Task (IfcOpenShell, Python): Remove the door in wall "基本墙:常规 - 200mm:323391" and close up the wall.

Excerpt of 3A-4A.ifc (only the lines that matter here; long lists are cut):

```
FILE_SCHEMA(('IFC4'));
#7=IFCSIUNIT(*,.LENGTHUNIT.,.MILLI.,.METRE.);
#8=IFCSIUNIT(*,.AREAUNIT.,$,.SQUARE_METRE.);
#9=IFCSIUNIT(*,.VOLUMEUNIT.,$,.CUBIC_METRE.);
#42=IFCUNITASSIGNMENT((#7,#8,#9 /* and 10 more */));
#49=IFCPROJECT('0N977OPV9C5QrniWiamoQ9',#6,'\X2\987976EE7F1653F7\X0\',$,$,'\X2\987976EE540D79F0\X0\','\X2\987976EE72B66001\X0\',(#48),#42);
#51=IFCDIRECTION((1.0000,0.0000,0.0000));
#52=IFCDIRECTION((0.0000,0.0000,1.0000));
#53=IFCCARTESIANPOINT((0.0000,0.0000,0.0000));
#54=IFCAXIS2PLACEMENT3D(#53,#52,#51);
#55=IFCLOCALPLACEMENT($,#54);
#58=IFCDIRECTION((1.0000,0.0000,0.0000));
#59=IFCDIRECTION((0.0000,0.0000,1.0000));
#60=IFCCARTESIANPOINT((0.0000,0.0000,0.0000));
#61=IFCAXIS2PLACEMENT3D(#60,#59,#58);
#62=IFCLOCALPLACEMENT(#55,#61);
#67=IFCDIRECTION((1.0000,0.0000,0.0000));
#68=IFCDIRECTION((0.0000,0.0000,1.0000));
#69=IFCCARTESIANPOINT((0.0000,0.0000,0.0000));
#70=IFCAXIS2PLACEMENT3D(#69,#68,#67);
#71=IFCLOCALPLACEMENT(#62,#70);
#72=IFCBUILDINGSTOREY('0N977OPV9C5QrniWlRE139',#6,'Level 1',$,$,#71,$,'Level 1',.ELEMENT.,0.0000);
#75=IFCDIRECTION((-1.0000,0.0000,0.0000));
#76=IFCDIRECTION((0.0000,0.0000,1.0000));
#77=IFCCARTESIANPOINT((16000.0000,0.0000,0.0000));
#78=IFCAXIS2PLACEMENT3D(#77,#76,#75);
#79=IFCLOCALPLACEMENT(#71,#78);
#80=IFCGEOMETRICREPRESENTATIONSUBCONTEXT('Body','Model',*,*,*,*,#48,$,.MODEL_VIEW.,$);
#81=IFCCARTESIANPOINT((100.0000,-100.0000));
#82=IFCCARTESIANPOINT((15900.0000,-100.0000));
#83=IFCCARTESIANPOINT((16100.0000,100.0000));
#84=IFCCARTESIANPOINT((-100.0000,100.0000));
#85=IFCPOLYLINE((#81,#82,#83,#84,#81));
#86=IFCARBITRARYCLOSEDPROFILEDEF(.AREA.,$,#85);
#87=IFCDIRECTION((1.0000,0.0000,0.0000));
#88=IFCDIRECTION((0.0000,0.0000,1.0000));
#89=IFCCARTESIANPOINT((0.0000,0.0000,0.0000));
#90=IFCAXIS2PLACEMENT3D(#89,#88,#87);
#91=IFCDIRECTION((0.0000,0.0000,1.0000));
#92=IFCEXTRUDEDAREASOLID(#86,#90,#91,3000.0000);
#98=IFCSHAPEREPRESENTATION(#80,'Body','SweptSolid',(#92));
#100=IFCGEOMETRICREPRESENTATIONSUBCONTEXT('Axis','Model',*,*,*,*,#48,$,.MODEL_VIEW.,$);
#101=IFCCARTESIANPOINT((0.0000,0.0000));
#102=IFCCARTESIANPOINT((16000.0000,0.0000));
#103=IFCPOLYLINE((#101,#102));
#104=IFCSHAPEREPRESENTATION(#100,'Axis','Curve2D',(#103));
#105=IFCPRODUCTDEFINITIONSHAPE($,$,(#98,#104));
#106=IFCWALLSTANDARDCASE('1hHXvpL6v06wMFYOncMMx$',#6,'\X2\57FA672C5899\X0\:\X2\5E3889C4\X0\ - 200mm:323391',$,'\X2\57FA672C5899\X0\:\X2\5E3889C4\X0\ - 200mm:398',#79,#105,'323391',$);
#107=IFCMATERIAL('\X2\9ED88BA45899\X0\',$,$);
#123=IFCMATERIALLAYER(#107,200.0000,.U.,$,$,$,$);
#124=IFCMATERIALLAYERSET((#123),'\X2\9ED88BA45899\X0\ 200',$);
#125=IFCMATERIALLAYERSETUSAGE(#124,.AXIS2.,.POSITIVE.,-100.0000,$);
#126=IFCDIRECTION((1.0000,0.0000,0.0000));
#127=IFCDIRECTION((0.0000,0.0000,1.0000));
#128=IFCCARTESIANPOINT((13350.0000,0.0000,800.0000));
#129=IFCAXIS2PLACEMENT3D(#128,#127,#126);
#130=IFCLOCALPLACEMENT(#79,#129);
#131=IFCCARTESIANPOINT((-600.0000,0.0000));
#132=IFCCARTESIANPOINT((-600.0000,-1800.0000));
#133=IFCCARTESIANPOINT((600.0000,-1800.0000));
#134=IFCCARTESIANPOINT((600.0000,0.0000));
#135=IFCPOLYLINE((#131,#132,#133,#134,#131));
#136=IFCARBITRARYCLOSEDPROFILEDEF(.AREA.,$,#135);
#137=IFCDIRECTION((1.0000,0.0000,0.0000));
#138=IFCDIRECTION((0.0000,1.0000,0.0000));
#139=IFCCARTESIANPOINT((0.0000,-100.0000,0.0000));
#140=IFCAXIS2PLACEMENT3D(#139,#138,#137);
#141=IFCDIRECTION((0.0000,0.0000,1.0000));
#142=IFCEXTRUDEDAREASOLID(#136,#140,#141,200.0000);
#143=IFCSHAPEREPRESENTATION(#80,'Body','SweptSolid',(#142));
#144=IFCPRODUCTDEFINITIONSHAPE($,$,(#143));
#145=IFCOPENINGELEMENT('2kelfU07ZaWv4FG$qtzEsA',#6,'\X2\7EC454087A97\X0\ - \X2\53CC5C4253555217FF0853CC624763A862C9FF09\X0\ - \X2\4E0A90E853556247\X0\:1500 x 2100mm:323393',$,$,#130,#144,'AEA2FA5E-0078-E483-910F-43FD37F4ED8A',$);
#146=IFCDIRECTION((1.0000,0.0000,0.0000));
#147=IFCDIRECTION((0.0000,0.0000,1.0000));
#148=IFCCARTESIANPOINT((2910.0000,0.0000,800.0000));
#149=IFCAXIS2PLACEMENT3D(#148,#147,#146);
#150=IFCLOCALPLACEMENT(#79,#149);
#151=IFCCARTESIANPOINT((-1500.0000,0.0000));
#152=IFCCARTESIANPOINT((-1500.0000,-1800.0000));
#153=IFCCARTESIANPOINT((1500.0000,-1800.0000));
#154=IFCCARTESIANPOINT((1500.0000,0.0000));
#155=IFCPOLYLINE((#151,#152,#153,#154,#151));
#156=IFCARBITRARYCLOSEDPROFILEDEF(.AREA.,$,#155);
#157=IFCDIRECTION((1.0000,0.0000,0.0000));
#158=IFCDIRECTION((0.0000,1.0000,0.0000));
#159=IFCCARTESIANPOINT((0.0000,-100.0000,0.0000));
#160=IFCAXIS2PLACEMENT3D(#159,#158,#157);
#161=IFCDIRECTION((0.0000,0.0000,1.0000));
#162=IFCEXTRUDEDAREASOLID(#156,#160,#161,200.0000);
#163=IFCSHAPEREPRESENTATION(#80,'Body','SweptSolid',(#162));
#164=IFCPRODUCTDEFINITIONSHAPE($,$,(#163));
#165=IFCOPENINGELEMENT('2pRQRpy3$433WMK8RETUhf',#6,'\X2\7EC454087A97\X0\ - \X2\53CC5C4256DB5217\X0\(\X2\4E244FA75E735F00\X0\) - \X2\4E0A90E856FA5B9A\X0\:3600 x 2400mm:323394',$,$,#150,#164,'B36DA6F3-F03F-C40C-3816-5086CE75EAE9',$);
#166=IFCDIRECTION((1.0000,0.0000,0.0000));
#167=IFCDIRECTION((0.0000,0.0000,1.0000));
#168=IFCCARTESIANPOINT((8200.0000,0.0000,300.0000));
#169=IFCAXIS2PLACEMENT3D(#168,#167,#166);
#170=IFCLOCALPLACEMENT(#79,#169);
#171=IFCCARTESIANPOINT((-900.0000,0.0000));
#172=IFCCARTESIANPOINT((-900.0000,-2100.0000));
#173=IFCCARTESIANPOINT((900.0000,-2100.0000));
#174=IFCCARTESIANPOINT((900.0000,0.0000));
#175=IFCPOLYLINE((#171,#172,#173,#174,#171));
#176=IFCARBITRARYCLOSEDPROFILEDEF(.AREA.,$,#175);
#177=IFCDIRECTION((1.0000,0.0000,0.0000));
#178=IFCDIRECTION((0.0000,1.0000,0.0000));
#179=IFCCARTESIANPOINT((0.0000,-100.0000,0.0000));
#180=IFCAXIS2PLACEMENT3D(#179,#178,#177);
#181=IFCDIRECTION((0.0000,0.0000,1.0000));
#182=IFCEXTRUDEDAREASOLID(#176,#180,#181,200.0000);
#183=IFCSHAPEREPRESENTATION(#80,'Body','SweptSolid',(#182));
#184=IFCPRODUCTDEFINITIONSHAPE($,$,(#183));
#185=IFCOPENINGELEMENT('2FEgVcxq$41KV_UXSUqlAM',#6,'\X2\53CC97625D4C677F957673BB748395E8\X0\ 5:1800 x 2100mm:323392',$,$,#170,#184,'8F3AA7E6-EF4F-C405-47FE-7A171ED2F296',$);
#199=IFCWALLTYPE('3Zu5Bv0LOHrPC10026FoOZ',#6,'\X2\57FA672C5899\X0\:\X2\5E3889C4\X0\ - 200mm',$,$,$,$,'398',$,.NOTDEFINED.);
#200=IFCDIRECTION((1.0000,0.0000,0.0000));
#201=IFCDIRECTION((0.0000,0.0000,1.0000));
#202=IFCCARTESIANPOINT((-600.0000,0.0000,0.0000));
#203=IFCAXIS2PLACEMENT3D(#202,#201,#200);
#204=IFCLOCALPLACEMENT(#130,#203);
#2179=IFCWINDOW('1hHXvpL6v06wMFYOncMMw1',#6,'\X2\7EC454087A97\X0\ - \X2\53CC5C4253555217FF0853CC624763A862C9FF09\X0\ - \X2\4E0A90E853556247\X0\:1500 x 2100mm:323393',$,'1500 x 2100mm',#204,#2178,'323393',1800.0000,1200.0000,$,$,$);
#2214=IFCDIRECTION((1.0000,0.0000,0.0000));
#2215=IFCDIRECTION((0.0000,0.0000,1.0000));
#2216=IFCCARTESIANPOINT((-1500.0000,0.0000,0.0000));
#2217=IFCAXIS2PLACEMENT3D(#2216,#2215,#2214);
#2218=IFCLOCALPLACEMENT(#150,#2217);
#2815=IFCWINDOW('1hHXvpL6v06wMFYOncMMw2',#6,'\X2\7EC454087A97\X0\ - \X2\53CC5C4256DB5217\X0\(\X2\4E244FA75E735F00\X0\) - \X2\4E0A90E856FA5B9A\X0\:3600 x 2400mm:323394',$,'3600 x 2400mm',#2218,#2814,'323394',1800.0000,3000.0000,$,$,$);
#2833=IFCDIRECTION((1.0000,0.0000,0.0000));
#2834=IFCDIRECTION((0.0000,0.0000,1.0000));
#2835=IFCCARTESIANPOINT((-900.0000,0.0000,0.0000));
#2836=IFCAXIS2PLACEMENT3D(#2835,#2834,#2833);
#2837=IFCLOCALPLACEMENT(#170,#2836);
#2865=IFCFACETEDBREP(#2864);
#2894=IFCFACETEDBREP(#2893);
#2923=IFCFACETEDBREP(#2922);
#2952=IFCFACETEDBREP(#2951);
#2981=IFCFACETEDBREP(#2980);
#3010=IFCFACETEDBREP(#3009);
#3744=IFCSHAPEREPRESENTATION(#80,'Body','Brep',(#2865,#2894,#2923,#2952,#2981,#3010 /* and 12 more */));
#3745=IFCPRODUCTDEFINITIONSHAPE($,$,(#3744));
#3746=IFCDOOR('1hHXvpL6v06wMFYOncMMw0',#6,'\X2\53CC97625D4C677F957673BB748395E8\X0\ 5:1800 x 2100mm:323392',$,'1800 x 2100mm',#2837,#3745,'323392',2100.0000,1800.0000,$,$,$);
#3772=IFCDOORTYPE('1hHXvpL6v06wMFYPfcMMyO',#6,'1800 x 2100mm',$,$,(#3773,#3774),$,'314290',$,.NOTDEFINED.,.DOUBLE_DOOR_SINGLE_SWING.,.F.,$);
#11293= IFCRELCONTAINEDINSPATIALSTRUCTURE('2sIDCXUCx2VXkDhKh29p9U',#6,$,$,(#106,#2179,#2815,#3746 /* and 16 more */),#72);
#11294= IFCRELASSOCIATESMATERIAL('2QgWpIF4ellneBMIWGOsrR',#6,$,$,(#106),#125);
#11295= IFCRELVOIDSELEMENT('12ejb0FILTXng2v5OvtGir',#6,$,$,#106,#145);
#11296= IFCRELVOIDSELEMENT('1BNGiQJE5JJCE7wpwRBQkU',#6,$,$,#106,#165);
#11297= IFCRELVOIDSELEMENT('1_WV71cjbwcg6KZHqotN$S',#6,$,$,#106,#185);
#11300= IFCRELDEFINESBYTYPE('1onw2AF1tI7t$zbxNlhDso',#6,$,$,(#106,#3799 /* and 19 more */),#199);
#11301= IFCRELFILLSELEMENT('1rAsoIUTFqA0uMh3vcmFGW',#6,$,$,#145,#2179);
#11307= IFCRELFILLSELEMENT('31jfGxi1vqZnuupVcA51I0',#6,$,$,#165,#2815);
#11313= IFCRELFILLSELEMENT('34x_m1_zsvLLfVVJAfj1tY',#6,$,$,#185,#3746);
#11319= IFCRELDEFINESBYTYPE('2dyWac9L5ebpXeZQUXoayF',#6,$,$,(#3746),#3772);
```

```python
import ifcopenshell
import ifcopenshell.api.feature
import ifcopenshell.api.root
import ifcopenshell.geom
import ifcopenshell.util.shape

model = ifcopenshell.open("3A-4A.ifc")
settings = ifcopenshell.geom.settings()


def volume(element):
    """Net volume in cubic metres, openings subtracted."""
    shape = ifcopenshell.geom.create_shape(settings, element)
    return ifcopenshell.util.shape.get_volume(shape.geometry)


door = model.by_guid("1hHXvpL6v06wMFYOncMMw0")
opening = door.FillsVoids[0].RelatingOpeningElement
wall = opening.VoidsElements[0].RelatingBuildingElement
before = volume(wall)

ifcopenshell.api.root.remove_product(model, product=door)
ifcopenshell.api.feature.remove_feature(model, feature=opening)

after = volume(wall)

print(f"wall volume {before:.3f} -> {after:.3f} m3")

model.write("3A-4A_edited.ifc")
```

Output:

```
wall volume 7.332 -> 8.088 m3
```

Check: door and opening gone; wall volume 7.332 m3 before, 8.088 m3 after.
